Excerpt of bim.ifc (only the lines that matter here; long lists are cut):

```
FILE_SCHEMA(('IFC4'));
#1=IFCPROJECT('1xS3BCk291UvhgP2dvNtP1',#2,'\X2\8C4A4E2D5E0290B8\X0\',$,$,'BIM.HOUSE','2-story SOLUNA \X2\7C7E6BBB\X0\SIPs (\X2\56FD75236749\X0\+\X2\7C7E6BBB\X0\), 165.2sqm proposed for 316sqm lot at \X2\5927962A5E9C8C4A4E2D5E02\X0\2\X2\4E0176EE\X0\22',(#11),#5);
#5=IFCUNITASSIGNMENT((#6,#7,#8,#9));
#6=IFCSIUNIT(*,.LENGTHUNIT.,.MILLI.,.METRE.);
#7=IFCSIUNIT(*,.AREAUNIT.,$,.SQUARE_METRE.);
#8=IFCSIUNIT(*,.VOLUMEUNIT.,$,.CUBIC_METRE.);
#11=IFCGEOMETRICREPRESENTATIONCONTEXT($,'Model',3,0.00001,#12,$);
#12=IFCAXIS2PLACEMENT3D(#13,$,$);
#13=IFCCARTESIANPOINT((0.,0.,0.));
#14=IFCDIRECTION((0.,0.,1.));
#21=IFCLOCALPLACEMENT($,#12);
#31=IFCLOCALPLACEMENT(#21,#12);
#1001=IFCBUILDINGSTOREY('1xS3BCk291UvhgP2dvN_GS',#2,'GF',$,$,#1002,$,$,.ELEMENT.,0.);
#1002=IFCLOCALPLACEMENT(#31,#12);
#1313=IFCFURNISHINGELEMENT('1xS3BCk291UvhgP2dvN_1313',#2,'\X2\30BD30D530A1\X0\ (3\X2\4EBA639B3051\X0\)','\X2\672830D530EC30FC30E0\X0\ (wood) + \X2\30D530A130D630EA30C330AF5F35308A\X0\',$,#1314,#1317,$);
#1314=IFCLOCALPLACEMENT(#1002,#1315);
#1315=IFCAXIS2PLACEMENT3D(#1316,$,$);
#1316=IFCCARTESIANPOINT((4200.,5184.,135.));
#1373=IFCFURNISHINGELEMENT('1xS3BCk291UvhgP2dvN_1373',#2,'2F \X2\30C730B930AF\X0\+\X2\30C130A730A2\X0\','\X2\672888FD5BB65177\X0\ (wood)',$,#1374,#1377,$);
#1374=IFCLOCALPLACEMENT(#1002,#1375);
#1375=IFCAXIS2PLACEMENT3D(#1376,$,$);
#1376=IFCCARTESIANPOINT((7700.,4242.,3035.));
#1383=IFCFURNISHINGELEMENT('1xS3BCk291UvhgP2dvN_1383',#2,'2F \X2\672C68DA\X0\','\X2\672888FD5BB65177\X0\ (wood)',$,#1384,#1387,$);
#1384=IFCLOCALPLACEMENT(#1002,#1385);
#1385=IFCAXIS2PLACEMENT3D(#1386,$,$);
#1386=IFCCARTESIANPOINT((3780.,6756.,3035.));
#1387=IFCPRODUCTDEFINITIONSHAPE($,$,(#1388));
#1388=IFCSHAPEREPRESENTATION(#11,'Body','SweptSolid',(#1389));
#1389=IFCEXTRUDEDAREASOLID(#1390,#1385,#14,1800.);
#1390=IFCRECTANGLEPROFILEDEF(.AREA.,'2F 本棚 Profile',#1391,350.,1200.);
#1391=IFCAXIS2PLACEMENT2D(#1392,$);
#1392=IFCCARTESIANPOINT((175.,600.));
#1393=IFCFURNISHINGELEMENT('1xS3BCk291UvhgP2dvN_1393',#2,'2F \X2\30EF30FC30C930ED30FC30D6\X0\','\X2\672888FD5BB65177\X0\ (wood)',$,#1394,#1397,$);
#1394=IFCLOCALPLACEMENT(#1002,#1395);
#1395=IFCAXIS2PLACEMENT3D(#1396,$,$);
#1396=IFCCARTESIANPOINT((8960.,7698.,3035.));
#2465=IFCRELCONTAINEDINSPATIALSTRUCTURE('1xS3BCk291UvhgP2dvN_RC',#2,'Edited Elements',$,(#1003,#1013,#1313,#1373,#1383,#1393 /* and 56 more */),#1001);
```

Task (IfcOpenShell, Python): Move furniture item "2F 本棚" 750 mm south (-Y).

```python
import ifcopenshell
import ifcopenshell.api.geometry
import ifcopenshell.util.placement
import ifcopenshell.util.unit

model = ifcopenshell.open("bim.ifc")
unit_scale = ifcopenshell.util.unit.calculate_unit_scale(model)

item = model.by_id(1383)
matrix = ifcopenshell.util.placement.get_local_placement(item.ObjectPlacement)
matrix[1, 3] -= 0.75 / unit_scale
ifcopenshell.api.geometry.edit_object_placement(model, product=item, matrix=matrix, is_si=False)

print(ifcopenshell.util.placement.get_local_placement(item.ObjectPlacement).round(3) + 0.0)

model.write("bim-out.ifc")
```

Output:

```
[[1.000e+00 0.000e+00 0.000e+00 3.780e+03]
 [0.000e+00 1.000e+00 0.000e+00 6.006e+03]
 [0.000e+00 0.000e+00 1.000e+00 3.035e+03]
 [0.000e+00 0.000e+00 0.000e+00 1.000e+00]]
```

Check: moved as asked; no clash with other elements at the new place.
